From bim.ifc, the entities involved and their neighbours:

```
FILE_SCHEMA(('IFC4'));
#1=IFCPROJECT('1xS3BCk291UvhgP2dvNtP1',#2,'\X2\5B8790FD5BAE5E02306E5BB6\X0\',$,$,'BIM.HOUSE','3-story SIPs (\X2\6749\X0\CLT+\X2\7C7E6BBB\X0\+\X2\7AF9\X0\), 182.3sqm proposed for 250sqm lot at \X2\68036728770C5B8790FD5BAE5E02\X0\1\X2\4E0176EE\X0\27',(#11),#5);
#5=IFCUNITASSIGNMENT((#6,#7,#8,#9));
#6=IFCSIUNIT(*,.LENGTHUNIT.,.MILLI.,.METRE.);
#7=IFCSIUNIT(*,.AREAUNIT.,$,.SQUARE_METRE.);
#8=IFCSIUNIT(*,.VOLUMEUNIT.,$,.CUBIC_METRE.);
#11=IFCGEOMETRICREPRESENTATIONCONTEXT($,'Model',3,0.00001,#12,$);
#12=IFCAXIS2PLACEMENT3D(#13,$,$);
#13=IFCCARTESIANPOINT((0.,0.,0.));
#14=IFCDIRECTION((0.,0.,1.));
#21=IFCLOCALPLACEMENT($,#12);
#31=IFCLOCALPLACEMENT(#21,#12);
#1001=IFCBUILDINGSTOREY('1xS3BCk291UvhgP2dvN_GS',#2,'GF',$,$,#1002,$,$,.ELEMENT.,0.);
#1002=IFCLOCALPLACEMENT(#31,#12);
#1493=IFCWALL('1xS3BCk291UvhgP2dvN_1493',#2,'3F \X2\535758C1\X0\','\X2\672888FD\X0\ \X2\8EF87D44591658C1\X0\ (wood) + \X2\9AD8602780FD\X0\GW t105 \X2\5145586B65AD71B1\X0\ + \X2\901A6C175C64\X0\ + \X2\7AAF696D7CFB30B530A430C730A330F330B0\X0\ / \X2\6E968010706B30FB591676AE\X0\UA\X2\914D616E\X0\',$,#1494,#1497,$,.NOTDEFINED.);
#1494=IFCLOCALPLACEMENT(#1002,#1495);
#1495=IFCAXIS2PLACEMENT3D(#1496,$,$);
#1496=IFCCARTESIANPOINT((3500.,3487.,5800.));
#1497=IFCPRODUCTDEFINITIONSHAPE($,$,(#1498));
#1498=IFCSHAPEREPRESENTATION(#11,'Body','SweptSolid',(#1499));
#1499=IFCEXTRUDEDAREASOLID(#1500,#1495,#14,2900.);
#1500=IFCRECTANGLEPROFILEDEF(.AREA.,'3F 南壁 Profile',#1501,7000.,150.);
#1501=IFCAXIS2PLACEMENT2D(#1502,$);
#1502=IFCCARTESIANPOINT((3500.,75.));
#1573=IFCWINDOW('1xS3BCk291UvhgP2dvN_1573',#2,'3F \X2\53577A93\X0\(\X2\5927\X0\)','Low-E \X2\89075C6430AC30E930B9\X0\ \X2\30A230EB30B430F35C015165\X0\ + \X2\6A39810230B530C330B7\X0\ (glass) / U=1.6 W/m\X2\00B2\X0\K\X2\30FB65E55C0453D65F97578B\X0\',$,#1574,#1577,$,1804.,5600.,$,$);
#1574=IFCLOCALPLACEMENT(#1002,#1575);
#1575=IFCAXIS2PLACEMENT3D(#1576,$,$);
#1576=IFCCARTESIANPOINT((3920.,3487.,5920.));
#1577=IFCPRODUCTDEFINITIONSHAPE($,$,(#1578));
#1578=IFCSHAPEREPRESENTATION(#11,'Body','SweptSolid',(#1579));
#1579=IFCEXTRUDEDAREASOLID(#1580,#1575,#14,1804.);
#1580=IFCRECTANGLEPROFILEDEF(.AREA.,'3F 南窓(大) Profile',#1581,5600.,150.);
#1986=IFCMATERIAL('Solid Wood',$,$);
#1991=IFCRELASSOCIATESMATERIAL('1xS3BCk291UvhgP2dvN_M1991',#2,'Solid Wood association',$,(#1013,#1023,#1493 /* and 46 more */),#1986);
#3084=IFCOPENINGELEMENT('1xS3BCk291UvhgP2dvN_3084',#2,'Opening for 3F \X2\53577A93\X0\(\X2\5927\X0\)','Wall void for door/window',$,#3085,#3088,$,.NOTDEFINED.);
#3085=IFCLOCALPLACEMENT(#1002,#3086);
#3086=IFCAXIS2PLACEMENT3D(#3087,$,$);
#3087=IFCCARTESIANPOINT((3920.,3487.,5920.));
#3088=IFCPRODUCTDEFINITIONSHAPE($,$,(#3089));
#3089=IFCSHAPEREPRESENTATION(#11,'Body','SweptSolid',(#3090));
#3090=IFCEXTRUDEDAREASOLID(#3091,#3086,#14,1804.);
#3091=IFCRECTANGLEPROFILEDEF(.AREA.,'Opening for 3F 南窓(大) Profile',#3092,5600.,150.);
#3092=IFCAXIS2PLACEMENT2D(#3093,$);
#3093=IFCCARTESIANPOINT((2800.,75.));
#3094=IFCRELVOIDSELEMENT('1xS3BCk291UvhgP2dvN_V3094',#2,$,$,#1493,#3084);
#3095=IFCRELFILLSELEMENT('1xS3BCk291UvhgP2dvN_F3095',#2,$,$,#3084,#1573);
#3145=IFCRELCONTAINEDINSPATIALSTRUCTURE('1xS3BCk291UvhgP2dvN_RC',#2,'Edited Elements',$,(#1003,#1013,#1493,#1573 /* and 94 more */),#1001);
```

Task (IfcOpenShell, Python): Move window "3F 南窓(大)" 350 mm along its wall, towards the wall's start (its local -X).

```python
import ifcopenshell
import ifcopenshell.api.geometry
import ifcopenshell.util.placement

model = ifcopenshell.open("bim.ifc")

window = model.by_guid("1xS3BCk291UvhgP2dvN_1573")
opening = window.FillsVoids[0].RelatingOpeningElement
wall = opening.VoidsElements[0].RelatingBuildingElement

wall_matrix = ifcopenshell.util.placement.get_local_placement(wall.ObjectPlacement)
shift = wall_matrix[:3, 0] * -350.0
before = ifcopenshell.util.placement.get_local_placement(window.ObjectPlacement)[:3, 3].copy()

# The window is not placed relative to its opening, so move both.
for product in (opening, window):
    matrix = ifcopenshell.util.placement.get_local_placement(product.ObjectPlacement)
    matrix[:3, 3] += shift
    ifcopenshell.api.geometry.edit_object_placement(model, product=product, matrix=matrix, is_si=False)

after = ifcopenshell.util.placement.get_local_placement(window.ObjectPlacement)[:3, 3]
print("window moved by", (after - before).round(3) + 0.0)

model.write("bim_updated.ifc")
```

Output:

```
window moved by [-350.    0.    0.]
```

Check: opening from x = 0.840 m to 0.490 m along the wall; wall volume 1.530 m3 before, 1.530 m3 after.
